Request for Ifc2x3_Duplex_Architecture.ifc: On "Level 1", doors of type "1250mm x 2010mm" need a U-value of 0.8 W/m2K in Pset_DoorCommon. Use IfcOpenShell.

First a look at what the model holds.

```python
import ifcopenshell
import ifcopenshell.util.element

model = ifcopenshell.open("Ifc2x3_Duplex_Architecture.ifc")
print(model.schema)
storey = next(s for s in model.by_type("IfcBuildingStorey") if s.Name == "Level 1")
doors = [e for e in ifcopenshell.util.element.get_decomposition(storey) if e.is_a("IfcDoor")]
seen = {}
for e in doors:
    element_type = ifcopenshell.util.element.get_type(e)
    key = (element_type.Name if element_type != e and element_type else None, ifcopenshell.util.element.get_pset(e, "Pset_DoorCommon", "ThermalTransmittance"))
    seen[key] = seen.get(key, 0) + 1
for (name, value), count in sorted(seen.items(), key=str):
    print(count, "x", name, "|", value)
```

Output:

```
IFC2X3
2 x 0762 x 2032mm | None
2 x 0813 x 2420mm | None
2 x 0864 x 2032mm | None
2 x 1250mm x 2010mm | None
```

```python
import ifcopenshell
import ifcopenshell.api.pset
import ifcopenshell.util.element

model = ifcopenshell.open("Ifc2x3_Duplex_Architecture.ifc")

storey = next(s for s in model.by_type("IfcBuildingStorey") if s.Name == "Level 1")
doors = [e for e in ifcopenshell.util.element.get_decomposition(storey) if e.is_a("IfcDoor")]

count = 0
for e in doors:
    element_type = ifcopenshell.util.element.get_type(e)
    if element_type in (None, e) or element_type.Name != "1250mm x 2010mm":
        continue
    # add_pset returns the element's existing set when there is one.
    pset = ifcopenshell.api.pset.add_pset(model, product=e, name="Pset_DoorCommon")
    ifcopenshell.api.pset.edit_pset(model, pset=pset, properties={"ThermalTransmittance": 0.8})
    count += 1

print(count, "doors updated")

model.write("Ifc2x3_Duplex_Architecture_updated.ifc")
```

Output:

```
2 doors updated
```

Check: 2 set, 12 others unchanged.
